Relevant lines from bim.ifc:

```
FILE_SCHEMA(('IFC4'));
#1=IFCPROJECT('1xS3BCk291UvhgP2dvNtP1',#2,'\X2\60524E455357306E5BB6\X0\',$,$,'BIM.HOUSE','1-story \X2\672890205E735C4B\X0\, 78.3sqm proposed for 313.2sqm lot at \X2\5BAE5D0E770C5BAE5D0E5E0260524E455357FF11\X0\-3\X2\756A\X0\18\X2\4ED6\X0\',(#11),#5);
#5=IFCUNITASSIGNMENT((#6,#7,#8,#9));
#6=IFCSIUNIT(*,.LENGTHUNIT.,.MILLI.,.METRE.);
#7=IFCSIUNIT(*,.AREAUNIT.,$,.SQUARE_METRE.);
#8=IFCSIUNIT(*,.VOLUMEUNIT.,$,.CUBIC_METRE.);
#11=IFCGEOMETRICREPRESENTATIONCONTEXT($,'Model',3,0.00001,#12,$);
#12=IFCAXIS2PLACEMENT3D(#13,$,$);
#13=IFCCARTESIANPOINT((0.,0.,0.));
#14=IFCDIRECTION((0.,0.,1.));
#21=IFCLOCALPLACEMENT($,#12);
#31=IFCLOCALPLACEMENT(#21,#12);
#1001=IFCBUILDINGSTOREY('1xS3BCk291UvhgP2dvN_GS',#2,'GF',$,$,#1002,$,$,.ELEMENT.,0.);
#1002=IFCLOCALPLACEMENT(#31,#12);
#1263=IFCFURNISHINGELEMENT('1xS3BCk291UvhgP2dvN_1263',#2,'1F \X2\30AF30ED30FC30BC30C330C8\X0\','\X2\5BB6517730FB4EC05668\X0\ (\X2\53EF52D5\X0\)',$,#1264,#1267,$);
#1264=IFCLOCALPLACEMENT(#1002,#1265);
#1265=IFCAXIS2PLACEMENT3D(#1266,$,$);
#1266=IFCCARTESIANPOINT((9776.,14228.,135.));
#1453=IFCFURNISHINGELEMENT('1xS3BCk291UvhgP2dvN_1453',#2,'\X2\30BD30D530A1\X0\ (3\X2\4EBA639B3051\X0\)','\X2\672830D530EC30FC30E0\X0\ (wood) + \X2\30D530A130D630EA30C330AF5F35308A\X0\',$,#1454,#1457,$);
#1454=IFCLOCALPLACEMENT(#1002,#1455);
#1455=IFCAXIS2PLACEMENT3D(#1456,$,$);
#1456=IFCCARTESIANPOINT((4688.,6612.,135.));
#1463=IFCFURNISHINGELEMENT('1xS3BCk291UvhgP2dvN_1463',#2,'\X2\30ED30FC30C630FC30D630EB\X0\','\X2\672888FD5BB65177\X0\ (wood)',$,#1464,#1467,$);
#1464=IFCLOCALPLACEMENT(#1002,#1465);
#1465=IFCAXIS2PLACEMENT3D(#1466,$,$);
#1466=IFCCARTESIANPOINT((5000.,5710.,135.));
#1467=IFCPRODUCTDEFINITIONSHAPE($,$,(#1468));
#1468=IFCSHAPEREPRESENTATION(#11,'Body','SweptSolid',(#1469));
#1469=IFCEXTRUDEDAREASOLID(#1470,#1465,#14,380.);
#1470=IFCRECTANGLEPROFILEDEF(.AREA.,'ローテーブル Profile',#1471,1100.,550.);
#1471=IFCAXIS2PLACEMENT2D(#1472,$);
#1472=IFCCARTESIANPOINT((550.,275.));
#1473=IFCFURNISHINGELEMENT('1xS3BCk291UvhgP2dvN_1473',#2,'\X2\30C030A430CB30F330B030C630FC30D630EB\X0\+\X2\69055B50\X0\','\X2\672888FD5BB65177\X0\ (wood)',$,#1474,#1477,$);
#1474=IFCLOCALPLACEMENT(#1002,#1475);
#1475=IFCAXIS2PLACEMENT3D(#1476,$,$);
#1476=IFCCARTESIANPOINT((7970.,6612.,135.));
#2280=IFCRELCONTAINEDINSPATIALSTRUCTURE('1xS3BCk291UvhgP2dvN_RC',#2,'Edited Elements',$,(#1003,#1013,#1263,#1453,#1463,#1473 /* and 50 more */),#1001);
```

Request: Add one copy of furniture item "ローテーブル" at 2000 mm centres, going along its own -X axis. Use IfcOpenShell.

```python
import ifcopenshell
import ifcopenshell.api.geometry
import ifcopenshell.api.root
import ifcopenshell.util.element
import ifcopenshell.util.placement
import ifcopenshell.util.unit

model = ifcopenshell.open("bim.ifc")
unit_scale = ifcopenshell.util.unit.calculate_unit_scale(model)


def reuse_history(source, copy):
    """copy_class also copies each property set's owner history, people and application; keep the originals."""
    for rel in copy.IsDefinedBy:
        if rel.is_a("IfcRelDefinesByProperties") and (history := rel.RelatingPropertyDefinition.OwnerHistory):
            rel.RelatingPropertyDefinition.OwnerHistory = source.OwnerHistory
            ifcopenshell.util.element.remove_deep2(model, history)


source = model.by_guid("1xS3BCk291UvhgP2dvN_1463")
base = ifcopenshell.util.placement.get_local_placement(source.ObjectPlacement)
step = -base[:3, 0] * 2 / unit_scale

for i in range(1, 2):
    copy = ifcopenshell.api.root.copy_class(model, product=source)
    copy.Representation = ifcopenshell.util.element.copy_deep(
        model, source.Representation, exclude=["IfcGeometricRepresentationContext", "IfcRepresentationMap"]
    )
    reuse_history(source, copy)
    matrix = base.copy()
    matrix[:3, 3] += i * step
    print("added at", matrix[:3, 3].round(3) + 0.0)
    ifcopenshell.api.geometry.edit_object_placement(model, product=copy, matrix=matrix, is_si=False)

model.write("bim_rev.ifc")
```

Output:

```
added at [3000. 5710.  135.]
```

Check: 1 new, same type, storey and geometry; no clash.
